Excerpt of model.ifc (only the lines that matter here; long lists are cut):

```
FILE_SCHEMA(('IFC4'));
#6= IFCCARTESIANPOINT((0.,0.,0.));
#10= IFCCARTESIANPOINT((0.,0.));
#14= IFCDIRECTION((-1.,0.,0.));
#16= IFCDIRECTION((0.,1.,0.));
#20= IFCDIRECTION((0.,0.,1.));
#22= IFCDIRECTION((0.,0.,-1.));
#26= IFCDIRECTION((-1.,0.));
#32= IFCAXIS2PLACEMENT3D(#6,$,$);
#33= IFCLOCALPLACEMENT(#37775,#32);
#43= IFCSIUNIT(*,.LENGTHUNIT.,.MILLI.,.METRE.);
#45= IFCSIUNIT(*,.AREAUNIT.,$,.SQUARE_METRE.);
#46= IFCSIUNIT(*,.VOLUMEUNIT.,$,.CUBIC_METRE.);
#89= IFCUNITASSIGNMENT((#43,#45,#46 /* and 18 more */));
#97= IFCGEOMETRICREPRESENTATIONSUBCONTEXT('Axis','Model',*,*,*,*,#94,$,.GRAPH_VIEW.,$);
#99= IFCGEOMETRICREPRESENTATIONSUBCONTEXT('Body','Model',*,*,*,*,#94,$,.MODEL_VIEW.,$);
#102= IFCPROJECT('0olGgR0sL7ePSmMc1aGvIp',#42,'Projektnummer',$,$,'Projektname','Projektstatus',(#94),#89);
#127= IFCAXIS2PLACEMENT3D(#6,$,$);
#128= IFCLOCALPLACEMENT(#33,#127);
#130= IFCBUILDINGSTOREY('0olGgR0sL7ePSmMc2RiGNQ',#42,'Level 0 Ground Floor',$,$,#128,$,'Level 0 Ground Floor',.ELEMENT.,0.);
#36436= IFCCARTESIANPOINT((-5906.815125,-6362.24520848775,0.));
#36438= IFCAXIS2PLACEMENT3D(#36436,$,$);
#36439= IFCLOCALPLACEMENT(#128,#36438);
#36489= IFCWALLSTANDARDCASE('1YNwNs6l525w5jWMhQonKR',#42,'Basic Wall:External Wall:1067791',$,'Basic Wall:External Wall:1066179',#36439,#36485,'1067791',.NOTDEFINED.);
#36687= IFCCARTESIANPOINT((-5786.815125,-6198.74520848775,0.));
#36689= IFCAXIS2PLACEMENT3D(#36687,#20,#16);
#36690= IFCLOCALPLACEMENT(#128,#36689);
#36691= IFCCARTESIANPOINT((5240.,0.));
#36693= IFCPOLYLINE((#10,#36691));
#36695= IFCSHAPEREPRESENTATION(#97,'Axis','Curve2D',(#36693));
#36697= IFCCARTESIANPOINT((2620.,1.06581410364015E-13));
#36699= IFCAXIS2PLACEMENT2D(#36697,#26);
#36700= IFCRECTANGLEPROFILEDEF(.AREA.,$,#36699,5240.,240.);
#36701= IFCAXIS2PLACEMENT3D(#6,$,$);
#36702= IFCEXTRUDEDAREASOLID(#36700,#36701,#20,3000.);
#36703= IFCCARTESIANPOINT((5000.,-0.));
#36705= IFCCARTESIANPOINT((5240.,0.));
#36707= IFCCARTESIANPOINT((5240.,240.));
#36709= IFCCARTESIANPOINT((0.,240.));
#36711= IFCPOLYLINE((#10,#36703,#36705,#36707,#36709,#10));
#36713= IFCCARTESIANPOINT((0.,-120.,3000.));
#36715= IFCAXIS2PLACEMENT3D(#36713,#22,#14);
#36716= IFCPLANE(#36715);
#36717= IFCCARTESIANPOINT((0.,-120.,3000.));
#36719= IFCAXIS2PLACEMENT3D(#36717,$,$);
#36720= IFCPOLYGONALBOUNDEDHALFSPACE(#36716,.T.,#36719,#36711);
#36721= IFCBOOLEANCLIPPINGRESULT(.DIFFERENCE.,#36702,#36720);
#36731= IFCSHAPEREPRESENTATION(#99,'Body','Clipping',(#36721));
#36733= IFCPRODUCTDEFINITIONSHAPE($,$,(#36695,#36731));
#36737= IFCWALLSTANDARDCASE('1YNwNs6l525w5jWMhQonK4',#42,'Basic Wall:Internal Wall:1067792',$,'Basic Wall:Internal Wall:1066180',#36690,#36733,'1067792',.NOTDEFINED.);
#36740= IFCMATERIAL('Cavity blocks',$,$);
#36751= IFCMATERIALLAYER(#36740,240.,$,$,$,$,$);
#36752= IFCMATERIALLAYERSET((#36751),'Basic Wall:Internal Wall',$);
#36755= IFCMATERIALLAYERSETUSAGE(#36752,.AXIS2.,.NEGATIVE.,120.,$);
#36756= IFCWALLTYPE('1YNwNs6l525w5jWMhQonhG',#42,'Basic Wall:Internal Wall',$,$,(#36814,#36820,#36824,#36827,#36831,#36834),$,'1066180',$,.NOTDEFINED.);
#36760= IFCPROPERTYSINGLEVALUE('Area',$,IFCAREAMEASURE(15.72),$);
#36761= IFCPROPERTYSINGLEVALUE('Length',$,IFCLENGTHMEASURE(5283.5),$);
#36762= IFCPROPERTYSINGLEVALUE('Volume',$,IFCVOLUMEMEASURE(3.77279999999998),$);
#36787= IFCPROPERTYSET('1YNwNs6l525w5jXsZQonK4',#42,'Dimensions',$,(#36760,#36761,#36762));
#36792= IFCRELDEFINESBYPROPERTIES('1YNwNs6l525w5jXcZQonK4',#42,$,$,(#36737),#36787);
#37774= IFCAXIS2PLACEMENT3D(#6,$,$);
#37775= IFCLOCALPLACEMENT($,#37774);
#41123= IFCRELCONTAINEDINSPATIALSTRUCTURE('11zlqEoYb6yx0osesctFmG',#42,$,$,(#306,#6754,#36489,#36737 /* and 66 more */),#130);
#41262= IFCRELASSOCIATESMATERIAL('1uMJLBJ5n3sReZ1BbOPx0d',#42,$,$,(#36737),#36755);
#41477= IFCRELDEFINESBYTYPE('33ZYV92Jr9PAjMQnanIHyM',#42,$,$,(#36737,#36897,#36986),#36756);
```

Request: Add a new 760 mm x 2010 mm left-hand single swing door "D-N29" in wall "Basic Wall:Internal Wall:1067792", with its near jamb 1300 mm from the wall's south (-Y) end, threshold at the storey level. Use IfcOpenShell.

```python
import numpy as np
import ifcopenshell
import ifcopenshell.api.feature
import ifcopenshell.api.geometry
import ifcopenshell.api.pset
import ifcopenshell.api.root
import ifcopenshell.api.spatial
import ifcopenshell.geom
import ifcopenshell.util.element
import ifcopenshell.util.placement
import ifcopenshell.util.representation
import ifcopenshell.util.shape
import ifcopenshell.util.unit

model = ifcopenshell.open("model.ifc")
unit_scale = ifcopenshell.util.unit.calculate_unit_scale(model)
area_scale = ifcopenshell.util.unit.calculate_unit_scale(model, "AREAUNIT")
volume_scale = ifcopenshell.util.unit.calculate_unit_scale(model, "VOLUMEUNIT")
settings = ifcopenshell.geom.settings()


def volume(element):
    """Net volume in cubic metres, openings subtracted."""
    shape = ifcopenshell.geom.create_shape(settings, element)
    return ifcopenshell.util.shape.get_volume(shape.geometry)


wall = model.by_id(36737)
storey = ifcopenshell.util.element.get_container(wall, ifc_class="IfcBuildingStorey")
context = ifcopenshell.util.representation.get_context(model, "Model", "Body", "MODEL_VIEW")
before = volume(wall)

width, height, from_end, sill = 0.76, 2.01, 1.3, 0.0  # metres

# The wall runs along its own X axis, and the end named is its -X end.
wall_shape = ifcopenshell.geom.create_shape(settings, wall)
x, y, z = ifcopenshell.util.shape.get_vertices(wall_shape.geometry).T
start = x.min() + from_end
face, thickness = float(y.min()), float(y.max() - y.min())
wall_matrix = ifcopenshell.util.placement.get_local_placement(wall.ObjectPlacement)
level = ifcopenshell.util.placement.get_local_placement(storey.ObjectPlacement)[2, 3]


def in_wall(x, y):
    """Placement at x, y metres in the wall's axes, at sill height."""
    matrix = wall_matrix.copy()
    matrix[:, 3] = wall_matrix @ np.array([x / unit_scale, y / unit_scale, 0.0, 1.0])
    matrix[2, 3] = level + sill / unit_scale
    return matrix


# Opening: a box that overshoots both wall faces by 50 mm.
opening = ifcopenshell.api.root.create_entity(model, ifc_class="IfcOpeningElement", predefined_type="OPENING")
box = ifcopenshell.api.geometry.add_wall_representation(
    model, context=context, length=width, height=height, thickness=thickness + 0.1
)
ifcopenshell.api.geometry.assign_representation(model, product=opening, representation=box)
ifcopenshell.api.geometry.edit_object_placement(model, product=opening, matrix=in_wall(start, face - 0.05), is_si=False)
ifcopenshell.api.feature.add_feature(model, feature=opening, element=wall)

door = ifcopenshell.api.root.create_entity(model, ifc_class="IfcDoor", name="D-N29", predefined_type="DOOR")
door.OverallWidth, door.OverallHeight = width / unit_scale, height / unit_scale
door.OperationType = "SINGLE_SWING_LEFT"
body = ifcopenshell.api.geometry.add_door_representation(
    model,
    context=context,
    overall_width=door.OverallWidth,
    overall_height=door.OverallHeight,
    operation_type="SINGLE_SWING_LEFT",
    lining_properties={"LiningDepth": thickness / unit_scale, "ThresholdDepth": thickness / unit_scale},
)
ifcopenshell.api.geometry.assign_representation(model, product=door, representation=body)
ifcopenshell.api.spatial.assign_container(model, products=[door], relating_structure=storey)
ifcopenshell.api.feature.add_filling(model, opening=opening, element=door)

# The lining spans the wall, so the door starts at the wall face.
ifcopenshell.api.geometry.edit_object_placement(model, product=door, matrix=in_wall(start, face), is_si=False)

after = volume(wall)

# Update the wall's stored quantities.
pset = model.by_id(ifcopenshell.util.element.get_pset(wall, "Dimensions", should_inherit=False)["id"])
ifcopenshell.api.pset.edit_pset(model, pset=pset, properties={
    "Area": model.create_entity("IfcAreaMeasure", after / thickness / area_scale),
    "Volume": model.create_entity("IfcVolumeMeasure", after / volume_scale),
})

print(f"wall volume {before:.3f} -> {after:.3f} m3")

model.write("model_updated.ifc")
```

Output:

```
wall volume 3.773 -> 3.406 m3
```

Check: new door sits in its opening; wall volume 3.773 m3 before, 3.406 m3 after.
